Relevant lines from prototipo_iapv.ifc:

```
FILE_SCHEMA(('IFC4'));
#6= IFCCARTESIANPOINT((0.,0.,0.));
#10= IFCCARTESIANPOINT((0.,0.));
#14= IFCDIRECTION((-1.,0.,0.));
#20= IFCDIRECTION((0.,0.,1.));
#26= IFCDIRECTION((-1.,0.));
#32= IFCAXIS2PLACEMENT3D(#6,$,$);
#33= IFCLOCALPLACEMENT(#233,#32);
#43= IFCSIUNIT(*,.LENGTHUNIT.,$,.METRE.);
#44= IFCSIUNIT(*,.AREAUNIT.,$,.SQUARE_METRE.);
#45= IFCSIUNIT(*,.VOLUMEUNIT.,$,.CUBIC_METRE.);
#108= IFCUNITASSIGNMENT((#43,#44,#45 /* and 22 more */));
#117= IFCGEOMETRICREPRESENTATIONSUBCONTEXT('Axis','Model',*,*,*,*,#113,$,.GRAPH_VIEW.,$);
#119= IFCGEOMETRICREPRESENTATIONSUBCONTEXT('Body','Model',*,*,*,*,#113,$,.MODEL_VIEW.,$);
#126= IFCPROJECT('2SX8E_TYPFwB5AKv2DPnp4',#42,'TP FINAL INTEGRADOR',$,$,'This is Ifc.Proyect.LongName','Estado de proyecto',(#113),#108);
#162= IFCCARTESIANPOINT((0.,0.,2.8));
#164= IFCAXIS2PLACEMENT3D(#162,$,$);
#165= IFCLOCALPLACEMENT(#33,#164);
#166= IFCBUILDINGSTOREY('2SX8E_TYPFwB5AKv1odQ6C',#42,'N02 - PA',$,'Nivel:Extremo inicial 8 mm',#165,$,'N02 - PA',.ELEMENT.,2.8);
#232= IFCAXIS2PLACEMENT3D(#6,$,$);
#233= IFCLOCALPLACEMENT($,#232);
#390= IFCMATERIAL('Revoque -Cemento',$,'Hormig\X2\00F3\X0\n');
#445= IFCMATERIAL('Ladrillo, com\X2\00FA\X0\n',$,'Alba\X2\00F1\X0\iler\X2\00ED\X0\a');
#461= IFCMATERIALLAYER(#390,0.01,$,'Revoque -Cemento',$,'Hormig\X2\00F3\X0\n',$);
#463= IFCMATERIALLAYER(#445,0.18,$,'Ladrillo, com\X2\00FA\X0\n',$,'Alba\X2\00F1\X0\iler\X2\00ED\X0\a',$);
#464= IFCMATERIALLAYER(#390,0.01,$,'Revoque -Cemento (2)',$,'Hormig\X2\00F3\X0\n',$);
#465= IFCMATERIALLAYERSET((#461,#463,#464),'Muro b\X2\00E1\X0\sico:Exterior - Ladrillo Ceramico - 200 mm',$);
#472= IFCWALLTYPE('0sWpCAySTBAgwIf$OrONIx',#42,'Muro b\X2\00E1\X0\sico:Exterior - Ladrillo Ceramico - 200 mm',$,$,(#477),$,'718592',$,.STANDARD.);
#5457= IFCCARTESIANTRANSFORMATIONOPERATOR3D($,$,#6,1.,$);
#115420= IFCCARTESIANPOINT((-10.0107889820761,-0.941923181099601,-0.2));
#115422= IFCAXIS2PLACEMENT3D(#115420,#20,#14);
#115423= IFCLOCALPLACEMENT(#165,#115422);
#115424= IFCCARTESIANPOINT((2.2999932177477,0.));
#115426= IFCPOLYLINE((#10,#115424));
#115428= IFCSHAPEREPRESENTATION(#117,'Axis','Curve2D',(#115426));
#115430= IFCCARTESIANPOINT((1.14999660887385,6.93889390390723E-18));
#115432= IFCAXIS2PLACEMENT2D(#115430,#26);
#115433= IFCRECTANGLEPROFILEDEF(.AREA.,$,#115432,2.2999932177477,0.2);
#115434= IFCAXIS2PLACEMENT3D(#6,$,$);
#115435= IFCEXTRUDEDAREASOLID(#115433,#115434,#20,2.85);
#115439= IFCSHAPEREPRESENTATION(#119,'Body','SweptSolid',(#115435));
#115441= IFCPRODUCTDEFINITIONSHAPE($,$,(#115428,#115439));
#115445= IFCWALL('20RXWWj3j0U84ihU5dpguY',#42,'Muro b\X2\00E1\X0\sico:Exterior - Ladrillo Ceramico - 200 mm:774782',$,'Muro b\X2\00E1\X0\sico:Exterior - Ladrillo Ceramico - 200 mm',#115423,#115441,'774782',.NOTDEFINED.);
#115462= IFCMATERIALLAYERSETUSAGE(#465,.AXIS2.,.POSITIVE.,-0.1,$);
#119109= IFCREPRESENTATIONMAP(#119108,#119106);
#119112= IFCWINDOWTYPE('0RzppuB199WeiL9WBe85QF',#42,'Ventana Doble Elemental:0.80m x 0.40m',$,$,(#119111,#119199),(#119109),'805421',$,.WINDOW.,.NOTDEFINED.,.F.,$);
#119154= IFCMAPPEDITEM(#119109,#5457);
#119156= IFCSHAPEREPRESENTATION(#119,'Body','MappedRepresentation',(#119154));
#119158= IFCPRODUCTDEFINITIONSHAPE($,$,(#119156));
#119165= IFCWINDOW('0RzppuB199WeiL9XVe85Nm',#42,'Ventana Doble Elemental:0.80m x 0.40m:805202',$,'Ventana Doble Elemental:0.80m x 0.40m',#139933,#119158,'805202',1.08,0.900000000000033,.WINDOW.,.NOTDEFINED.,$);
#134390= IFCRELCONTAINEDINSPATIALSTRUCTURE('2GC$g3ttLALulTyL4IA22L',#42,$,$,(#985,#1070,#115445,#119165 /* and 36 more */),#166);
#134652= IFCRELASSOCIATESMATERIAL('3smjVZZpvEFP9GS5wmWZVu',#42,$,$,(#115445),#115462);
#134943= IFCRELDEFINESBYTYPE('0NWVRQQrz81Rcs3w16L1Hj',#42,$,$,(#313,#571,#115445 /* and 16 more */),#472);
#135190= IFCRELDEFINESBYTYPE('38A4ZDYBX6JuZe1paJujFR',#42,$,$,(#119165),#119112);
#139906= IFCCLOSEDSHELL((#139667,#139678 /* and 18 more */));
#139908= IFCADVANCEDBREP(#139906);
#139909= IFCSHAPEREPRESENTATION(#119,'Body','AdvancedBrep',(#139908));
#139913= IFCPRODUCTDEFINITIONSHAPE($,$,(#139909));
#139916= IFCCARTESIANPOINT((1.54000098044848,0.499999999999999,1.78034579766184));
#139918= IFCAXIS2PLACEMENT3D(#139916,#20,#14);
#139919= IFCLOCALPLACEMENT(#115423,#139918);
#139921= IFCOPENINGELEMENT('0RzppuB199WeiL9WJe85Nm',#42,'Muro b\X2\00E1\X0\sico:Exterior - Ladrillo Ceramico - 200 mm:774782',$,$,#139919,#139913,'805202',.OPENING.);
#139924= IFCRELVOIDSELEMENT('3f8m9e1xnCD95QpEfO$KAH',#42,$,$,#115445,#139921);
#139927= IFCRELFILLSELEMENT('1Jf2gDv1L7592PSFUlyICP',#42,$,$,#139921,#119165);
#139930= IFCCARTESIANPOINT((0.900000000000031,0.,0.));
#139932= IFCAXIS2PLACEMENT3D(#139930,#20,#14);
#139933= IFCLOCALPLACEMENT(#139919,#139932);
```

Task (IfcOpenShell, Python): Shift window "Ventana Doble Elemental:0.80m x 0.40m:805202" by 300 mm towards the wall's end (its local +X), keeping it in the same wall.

```python
import ifcopenshell
import ifcopenshell.api.geometry
import ifcopenshell.util.placement
import ifcopenshell.util.unit

model = ifcopenshell.open("prototipo_iapv.ifc")
unit_scale = ifcopenshell.util.unit.calculate_unit_scale(model)

window = model.by_guid("0RzppuB199WeiL9XVe85Nm")
opening = window.FillsVoids[0].RelatingOpeningElement
wall = opening.VoidsElements[0].RelatingBuildingElement

wall_matrix = ifcopenshell.util.placement.get_local_placement(wall.ObjectPlacement)
shift = wall_matrix[:3, 0] * 0.3 / unit_scale
before = ifcopenshell.util.placement.get_local_placement(window.ObjectPlacement)[:3, 3].copy()

# The window is placed relative to its opening, so it follows when the opening moves.
matrix = ifcopenshell.util.placement.get_local_placement(opening.ObjectPlacement)
matrix[:3, 3] += shift
ifcopenshell.api.geometry.edit_object_placement(
    model, product=opening, matrix=matrix, is_si=False, should_transform_children=True
)

after = ifcopenshell.util.placement.get_local_placement(window.ObjectPlacement)[:3, 3]
print("window moved by", (after - before).round(3) + 0.0)

model.write("prototipo_iapv_updated.ifc")
```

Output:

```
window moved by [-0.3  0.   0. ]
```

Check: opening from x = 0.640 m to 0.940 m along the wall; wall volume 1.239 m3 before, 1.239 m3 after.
